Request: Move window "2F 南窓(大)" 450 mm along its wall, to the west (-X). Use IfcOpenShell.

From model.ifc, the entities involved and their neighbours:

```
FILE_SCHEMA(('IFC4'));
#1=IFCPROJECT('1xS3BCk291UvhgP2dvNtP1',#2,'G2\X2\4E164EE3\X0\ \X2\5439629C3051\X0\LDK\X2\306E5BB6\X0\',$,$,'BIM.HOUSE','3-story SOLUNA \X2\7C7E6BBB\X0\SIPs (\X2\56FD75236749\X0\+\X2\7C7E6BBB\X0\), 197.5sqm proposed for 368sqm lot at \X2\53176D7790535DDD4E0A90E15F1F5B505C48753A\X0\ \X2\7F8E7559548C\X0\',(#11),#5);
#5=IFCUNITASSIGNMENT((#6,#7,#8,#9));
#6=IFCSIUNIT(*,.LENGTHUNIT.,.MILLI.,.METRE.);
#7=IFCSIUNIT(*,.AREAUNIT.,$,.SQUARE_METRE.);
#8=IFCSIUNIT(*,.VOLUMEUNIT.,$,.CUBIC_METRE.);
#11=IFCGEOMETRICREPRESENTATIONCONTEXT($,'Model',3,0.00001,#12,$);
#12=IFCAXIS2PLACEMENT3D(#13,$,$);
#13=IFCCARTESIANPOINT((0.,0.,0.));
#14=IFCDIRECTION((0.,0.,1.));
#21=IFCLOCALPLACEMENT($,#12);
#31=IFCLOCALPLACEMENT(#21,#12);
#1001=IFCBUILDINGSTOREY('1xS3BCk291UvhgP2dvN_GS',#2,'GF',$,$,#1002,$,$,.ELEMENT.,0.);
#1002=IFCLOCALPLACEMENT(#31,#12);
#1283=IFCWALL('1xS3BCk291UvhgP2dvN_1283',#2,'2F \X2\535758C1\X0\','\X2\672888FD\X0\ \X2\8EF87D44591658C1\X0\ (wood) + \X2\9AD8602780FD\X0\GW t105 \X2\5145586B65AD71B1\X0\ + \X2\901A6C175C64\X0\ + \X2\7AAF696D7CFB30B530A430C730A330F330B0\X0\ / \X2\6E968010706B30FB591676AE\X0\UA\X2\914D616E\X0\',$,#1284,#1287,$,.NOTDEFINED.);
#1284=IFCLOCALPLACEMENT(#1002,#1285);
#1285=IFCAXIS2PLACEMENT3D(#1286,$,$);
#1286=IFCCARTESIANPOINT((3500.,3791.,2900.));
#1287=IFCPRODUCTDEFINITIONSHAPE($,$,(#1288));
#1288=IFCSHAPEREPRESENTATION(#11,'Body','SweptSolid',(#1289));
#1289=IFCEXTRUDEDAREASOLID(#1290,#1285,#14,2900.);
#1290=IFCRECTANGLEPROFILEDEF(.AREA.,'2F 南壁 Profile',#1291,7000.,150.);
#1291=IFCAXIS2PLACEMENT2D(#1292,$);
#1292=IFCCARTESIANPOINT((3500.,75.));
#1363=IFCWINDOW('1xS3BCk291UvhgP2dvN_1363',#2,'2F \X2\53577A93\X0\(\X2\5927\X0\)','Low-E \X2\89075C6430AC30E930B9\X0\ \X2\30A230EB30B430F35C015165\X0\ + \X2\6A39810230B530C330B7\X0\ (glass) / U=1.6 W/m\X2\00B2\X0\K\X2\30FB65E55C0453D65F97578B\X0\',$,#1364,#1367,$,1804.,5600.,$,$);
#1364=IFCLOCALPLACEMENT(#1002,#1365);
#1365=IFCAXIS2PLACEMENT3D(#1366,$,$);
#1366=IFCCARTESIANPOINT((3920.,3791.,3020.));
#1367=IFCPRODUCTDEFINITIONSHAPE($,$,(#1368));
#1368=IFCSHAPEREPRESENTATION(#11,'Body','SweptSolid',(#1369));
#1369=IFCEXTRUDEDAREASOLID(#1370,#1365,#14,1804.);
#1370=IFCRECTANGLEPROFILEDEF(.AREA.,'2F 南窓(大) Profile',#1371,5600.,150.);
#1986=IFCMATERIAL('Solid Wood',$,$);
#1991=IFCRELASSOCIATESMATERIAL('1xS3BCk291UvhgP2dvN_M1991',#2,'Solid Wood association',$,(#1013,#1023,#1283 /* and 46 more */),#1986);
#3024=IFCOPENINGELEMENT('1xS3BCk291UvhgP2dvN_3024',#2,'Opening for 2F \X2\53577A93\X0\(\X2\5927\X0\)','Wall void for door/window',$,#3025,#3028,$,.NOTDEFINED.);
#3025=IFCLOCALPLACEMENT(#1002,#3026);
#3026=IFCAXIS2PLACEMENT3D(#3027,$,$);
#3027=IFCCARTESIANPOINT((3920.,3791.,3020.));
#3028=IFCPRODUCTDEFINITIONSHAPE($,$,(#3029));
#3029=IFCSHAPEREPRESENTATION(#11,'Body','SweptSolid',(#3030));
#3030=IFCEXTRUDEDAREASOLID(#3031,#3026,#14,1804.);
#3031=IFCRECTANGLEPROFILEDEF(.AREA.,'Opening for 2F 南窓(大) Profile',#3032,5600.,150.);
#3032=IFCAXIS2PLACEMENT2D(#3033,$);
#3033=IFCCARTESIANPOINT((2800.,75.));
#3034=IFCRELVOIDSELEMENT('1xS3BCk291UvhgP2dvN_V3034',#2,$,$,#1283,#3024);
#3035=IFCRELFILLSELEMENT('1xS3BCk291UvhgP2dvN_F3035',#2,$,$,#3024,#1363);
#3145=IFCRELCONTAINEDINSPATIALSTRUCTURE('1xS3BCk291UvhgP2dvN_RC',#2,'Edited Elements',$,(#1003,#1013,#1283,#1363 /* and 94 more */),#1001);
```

```python
import ifcopenshell
import ifcopenshell.api.geometry
import ifcopenshell.util.placement

model = ifcopenshell.open("model.ifc")

window = model.by_guid("1xS3BCk291UvhgP2dvN_1363")
opening = window.FillsVoids[0].RelatingOpeningElement
wall = opening.VoidsElements[0].RelatingBuildingElement

wall_matrix = ifcopenshell.util.placement.get_local_placement(wall.ObjectPlacement)
shift = wall_matrix[:3, 0] * -450.0
before = ifcopenshell.util.placement.get_local_placement(window.ObjectPlacement)[:3, 3].copy()

# The window is not placed relative to its opening, so move both.
for product in (opening, window):
    matrix = ifcopenshell.util.placement.get_local_placement(product.ObjectPlacement)
    matrix[:3, 3] += shift
    ifcopenshell.api.geometry.edit_object_placement(model, product=product, matrix=matrix, is_si=False)

after = ifcopenshell.util.placement.get_local_placement(window.ObjectPlacement)[:3, 3]
print("window moved by", (after - before).round(3) + 0.0)

model.write("model_edited.ifc")
```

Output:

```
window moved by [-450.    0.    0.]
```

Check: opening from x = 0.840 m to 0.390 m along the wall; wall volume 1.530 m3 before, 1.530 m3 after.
